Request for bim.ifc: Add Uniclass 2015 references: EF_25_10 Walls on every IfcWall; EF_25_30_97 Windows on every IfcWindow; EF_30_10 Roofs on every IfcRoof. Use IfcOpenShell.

First a look at what the model holds.

```python
import ifcopenshell

model = ifcopenshell.open("bim.ifc")
print(model.schema)
print("classifications:", [c.Name for c in model.by_type("IfcClassification")])
for ifc_class in ("IfcDoor", "IfcRoof", "IfcStair", "IfcWall", "IfcWindow"):
    print(ifc_class, len(model.by_type(ifc_class)))
```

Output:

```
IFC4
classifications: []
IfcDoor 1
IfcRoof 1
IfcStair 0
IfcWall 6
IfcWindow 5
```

```python
import ifcopenshell
import ifcopenshell.api.classification

model = ifcopenshell.open("bim.ifc")

system = ifcopenshell.api.classification.add_classification(model, classification="Uniclass 2015")

codes = {
    "IfcWall": ("EF_25_10", "Walls"),
    "IfcWindow": ("EF_25_30_97", "Windows"),
    "IfcRoof": ("EF_30_10", "Roofs"),
}
for ifc_class, (code, name) in codes.items():
    products = model.by_type(ifc_class)
    ifcopenshell.api.classification.add_reference(
        model, products=products, classification=system, identification=code, name=name
    )
    print(code, len(products))

model.write("bim_v2.ifc")
```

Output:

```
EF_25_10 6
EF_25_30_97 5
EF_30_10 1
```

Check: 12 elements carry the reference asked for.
